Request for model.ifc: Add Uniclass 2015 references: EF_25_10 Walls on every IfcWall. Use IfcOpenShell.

First a look at what the model holds.

```python
import ifcopenshell

model = ifcopenshell.open("model.ifc")
print(model.schema)
print("classifications:", [c.Name for c in model.by_type("IfcClassification")])
for ifc_class in ("IfcDoor", "IfcRoof", "IfcStair", "IfcWall", "IfcWindow"):
    print(ifc_class, len(model.by_type(ifc_class)))
```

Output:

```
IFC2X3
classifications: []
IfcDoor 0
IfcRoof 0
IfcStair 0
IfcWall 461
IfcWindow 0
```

```python
import ifcopenshell
import ifcopenshell.api.classification

model = ifcopenshell.open("model.ifc")

# IFC2X3 requires Source and Edition and has no link from the project to the system.
system = model.create_entity("IfcClassification", Source="NBS", Edition="2015", Name="Uniclass 2015")

codes = {
    "IfcWall": ("EF_25_10", "Walls"),
}
for ifc_class, (code, name) in codes.items():
    products = model.by_type(ifc_class)
    ifcopenshell.api.classification.add_reference(
        model, products=products, classification=system, identification=code, name=name
    )
    print(code, len(products))

model.write("model_edited.ifc")
```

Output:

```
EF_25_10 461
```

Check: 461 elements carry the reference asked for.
